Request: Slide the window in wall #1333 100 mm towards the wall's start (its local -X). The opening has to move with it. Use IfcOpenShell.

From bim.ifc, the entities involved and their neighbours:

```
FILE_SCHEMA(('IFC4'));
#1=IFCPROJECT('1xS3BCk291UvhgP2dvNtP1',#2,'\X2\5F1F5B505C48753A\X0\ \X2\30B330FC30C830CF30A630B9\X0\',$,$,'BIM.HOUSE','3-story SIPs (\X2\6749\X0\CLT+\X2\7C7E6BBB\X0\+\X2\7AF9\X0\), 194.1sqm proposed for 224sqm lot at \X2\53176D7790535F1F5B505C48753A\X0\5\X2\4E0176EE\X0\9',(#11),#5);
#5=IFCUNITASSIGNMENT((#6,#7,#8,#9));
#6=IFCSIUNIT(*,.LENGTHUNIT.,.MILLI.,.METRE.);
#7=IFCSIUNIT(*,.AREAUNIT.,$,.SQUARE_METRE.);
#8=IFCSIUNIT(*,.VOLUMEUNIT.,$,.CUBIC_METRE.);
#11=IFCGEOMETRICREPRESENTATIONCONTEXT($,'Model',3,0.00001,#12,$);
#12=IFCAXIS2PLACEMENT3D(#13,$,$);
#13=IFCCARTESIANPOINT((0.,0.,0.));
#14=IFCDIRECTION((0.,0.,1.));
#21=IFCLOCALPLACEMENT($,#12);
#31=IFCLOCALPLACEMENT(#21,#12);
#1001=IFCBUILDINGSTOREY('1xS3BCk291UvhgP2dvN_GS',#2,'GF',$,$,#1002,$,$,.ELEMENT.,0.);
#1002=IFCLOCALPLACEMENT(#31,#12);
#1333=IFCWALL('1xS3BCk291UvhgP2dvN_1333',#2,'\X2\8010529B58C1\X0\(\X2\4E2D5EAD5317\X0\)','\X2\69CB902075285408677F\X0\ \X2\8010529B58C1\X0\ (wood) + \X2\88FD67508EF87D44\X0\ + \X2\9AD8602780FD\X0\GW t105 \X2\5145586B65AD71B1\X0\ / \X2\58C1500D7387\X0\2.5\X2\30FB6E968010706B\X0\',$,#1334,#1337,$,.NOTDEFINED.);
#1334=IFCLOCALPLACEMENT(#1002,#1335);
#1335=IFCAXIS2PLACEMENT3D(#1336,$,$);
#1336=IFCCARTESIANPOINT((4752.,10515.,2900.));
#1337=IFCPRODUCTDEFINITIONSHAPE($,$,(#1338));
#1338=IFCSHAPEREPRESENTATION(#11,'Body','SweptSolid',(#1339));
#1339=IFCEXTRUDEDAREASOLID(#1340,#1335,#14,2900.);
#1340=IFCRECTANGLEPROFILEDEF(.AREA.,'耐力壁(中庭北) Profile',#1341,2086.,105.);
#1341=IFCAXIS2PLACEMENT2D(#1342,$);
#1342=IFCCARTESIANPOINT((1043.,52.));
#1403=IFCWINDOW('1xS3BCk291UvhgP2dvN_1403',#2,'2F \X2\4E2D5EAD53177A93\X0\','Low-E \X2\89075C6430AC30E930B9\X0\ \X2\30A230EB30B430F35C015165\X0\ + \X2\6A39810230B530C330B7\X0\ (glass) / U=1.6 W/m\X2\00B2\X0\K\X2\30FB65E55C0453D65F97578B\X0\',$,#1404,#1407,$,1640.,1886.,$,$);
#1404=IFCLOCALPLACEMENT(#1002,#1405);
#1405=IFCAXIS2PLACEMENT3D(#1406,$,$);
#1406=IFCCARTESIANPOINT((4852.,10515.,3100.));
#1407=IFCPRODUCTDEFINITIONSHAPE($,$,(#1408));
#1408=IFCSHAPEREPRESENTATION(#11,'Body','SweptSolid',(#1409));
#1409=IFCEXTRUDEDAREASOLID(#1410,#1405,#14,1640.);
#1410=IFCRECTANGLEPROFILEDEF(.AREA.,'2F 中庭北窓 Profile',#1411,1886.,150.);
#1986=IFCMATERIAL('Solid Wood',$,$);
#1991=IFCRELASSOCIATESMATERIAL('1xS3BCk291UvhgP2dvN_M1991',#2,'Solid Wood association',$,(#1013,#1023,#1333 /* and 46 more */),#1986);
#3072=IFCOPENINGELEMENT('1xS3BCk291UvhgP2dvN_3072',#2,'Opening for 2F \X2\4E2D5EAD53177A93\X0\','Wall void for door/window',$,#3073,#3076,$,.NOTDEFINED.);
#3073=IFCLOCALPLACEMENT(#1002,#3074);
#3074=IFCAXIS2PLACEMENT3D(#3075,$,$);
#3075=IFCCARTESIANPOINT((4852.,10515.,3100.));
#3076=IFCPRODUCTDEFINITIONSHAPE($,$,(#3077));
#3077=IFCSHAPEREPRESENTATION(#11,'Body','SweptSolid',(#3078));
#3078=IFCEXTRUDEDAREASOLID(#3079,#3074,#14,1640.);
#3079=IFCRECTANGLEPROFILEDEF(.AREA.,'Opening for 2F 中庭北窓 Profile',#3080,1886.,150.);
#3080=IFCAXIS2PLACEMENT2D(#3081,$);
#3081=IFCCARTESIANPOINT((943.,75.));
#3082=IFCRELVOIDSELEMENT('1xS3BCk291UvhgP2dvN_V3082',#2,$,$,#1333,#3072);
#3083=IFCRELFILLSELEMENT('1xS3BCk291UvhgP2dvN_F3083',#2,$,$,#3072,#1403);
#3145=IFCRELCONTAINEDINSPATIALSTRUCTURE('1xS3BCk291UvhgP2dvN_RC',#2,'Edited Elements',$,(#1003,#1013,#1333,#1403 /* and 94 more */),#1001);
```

```python
import ifcopenshell
import ifcopenshell.api.geometry
import ifcopenshell.util.placement

model = ifcopenshell.open("bim.ifc")

window = model.by_guid("1xS3BCk291UvhgP2dvN_1403")
opening = window.FillsVoids[0].RelatingOpeningElement
wall = opening.VoidsElements[0].RelatingBuildingElement

wall_matrix = ifcopenshell.util.placement.get_local_placement(wall.ObjectPlacement)
shift = wall_matrix[:3, 0] * -100.0
before = ifcopenshell.util.placement.get_local_placement(window.ObjectPlacement)[:3, 3].copy()

# The window is not placed relative to its opening, so move both.
for product in (opening, window):
    matrix = ifcopenshell.util.placement.get_local_placement(product.ObjectPlacement)
    matrix[:3, 3] += shift
    ifcopenshell.api.geometry.edit_object_placement(model, product=product, matrix=matrix, is_si=False)

after = ifcopenshell.util.placement.get_local_placement(window.ObjectPlacement)[:3, 3]
print("window moved by", (after - before).round(3) + 0.0)

model.write("bim-out.ifc")
```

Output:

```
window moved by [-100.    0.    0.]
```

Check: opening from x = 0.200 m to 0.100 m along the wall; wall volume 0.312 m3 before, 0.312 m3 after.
